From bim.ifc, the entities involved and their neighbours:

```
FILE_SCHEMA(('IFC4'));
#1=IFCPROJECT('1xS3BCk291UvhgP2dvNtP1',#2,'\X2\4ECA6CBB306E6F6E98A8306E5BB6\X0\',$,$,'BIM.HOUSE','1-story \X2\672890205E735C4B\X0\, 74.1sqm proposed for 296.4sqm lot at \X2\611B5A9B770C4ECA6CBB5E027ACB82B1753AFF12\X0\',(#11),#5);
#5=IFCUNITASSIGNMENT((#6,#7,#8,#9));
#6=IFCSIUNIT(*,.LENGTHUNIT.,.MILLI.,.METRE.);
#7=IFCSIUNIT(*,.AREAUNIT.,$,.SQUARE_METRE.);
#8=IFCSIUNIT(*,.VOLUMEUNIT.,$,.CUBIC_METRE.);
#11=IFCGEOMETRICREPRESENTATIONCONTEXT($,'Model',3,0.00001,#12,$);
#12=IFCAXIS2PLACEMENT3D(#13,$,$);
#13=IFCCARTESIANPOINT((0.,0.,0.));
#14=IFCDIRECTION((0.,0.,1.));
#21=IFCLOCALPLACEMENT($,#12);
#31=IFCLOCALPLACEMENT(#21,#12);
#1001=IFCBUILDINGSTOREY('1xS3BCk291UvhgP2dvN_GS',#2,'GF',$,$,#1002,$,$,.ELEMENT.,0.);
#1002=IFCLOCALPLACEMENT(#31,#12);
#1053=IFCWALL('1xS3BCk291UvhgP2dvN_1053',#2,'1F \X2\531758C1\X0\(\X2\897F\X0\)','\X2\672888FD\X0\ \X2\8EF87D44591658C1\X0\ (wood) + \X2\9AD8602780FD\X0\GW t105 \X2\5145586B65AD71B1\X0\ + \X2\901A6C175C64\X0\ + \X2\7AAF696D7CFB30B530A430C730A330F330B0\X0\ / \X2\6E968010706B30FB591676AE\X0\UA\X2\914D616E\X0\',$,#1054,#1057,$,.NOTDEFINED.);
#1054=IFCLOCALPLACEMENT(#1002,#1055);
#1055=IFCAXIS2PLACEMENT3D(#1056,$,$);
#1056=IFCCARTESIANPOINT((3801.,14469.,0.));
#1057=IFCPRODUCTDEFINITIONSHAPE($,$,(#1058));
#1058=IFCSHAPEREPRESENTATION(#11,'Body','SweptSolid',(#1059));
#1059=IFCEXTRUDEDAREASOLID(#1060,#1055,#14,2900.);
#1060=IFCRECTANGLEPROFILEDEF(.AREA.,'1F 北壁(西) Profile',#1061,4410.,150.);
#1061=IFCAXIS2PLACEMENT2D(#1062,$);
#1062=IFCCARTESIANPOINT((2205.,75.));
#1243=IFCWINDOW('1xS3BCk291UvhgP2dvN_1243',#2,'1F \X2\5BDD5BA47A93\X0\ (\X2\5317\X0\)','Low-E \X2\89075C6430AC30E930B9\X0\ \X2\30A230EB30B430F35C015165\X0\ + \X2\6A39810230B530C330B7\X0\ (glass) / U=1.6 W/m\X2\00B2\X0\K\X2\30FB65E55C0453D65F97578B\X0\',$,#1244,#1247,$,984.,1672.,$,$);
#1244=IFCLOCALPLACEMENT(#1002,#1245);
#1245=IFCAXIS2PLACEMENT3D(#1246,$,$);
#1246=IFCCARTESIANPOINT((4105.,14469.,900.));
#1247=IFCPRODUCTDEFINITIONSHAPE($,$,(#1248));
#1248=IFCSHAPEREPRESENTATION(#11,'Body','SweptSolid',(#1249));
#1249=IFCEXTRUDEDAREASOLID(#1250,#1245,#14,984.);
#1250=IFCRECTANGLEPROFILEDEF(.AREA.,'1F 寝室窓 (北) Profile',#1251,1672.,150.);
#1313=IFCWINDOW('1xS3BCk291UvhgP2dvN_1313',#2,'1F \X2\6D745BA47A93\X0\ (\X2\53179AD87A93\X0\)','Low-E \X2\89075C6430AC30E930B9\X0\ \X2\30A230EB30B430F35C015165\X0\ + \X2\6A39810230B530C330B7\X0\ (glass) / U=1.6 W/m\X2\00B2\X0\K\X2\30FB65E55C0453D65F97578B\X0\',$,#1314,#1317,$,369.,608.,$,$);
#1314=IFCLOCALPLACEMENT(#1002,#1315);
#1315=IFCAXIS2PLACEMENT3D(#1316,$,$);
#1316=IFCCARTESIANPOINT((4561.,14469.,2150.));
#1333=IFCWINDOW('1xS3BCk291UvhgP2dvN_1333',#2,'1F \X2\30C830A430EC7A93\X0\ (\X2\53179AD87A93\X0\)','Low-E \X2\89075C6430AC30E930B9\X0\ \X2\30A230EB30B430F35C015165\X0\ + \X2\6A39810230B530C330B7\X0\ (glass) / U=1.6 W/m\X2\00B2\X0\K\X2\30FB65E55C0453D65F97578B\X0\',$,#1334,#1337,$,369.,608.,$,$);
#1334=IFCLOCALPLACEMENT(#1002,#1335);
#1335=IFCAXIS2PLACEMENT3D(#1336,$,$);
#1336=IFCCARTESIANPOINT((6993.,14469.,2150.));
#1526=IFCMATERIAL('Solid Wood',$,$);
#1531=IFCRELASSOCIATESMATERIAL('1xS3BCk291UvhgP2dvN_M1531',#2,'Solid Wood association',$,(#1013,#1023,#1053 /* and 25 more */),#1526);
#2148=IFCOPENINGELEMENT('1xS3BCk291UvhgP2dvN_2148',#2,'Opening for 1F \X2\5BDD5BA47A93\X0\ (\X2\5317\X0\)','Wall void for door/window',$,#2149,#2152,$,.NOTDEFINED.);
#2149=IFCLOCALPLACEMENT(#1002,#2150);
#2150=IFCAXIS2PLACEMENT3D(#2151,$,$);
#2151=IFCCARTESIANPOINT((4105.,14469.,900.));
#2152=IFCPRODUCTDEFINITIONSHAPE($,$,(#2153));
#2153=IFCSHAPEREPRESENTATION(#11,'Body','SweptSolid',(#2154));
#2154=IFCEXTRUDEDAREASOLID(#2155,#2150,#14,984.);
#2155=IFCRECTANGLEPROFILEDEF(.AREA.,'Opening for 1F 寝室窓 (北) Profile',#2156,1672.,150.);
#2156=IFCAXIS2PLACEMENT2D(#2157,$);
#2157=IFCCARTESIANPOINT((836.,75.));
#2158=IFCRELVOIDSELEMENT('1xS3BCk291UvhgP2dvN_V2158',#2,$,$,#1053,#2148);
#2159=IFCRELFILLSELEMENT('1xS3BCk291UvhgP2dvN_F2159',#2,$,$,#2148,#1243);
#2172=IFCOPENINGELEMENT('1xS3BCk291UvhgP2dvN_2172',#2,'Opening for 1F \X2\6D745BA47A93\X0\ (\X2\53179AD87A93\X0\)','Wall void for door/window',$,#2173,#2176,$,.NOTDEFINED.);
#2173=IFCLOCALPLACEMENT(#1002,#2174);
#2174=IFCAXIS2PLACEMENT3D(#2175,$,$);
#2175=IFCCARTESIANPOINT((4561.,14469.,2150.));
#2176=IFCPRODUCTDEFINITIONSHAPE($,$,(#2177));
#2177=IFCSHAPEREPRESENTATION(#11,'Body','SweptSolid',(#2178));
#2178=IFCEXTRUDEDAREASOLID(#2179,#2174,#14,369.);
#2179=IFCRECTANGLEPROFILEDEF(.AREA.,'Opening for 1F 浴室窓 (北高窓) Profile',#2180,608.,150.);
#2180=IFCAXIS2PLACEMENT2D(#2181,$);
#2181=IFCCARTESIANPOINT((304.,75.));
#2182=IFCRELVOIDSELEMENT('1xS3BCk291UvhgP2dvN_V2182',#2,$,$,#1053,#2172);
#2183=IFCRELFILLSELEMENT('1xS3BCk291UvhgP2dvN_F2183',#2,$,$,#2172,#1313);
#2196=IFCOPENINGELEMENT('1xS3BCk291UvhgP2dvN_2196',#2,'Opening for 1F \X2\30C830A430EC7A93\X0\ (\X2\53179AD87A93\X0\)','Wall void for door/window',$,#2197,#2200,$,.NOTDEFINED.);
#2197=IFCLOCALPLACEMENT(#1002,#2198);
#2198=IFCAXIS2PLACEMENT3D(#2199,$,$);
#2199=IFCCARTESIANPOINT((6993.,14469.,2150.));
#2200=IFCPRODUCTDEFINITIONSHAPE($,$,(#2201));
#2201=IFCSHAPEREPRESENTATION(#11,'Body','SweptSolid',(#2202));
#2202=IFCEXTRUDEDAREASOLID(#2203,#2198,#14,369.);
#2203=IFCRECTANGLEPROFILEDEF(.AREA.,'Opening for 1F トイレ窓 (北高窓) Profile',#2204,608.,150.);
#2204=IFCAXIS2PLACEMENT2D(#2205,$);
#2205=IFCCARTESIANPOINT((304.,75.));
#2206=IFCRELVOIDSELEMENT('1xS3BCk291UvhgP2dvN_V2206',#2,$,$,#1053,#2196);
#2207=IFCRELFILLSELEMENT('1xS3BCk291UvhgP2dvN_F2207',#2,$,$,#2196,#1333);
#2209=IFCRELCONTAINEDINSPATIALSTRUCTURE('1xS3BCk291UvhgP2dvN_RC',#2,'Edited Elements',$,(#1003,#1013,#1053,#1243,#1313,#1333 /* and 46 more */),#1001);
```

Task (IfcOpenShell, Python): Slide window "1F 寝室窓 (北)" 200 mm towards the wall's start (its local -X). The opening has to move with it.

```python
import ifcopenshell
import ifcopenshell.api.geometry
import ifcopenshell.util.placement
import ifcopenshell.util.unit

model = ifcopenshell.open("bim.ifc")
unit_scale = ifcopenshell.util.unit.calculate_unit_scale(model)

window = model.by_guid("1xS3BCk291UvhgP2dvN_1243")
opening = window.FillsVoids[0].RelatingOpeningElement
wall = opening.VoidsElements[0].RelatingBuildingElement

wall_matrix = ifcopenshell.util.placement.get_local_placement(wall.ObjectPlacement)
shift = wall_matrix[:3, 0] * -0.2 / unit_scale
before = ifcopenshell.util.placement.get_local_placement(window.ObjectPlacement)[:3, 3].copy()

# The window is not placed relative to its opening, so move both.
for product in (opening, window):
    matrix = ifcopenshell.util.placement.get_local_placement(product.ObjectPlacement)
    matrix[:3, 3] += shift
    ifcopenshell.api.geometry.edit_object_placement(model, product=product, matrix=matrix, is_si=False)

after = ifcopenshell.util.placement.get_local_placement(window.ObjectPlacement)[:3, 3]
print("window moved by", (after - before).round(3) + 0.0)

model.write("bim_v2.ifc")
```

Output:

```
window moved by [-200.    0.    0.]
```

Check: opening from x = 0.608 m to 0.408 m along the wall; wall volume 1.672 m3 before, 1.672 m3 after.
